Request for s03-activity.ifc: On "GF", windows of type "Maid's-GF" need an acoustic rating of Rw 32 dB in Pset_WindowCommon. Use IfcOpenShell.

First a look at what the model holds.

```python
import ifcopenshell
import ifcopenshell.util.element

model = ifcopenshell.open("s03-activity.ifc")
print(model.schema)
storey = next(s for s in model.by_type("IfcBuildingStorey") if s.Name == "GF")
windows = [e for e in ifcopenshell.util.element.get_decomposition(storey) if e.is_a("IfcWindow")]
seen = {}
for e in windows:
    element_type = ifcopenshell.util.element.get_type(e)
    key = (element_type.Name if element_type != e and element_type else None, ifcopenshell.util.element.get_pset(e, "Pset_WindowCommon", "AcousticRating"))
    seen[key] = seen.get(key, 0) + 1
for (name, value), count in sorted(seen.items(), key=str):
    print(count, "x", name, "|", value)
```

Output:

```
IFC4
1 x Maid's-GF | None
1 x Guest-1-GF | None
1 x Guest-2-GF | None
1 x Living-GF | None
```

```python
import ifcopenshell
import ifcopenshell.api.pset
import ifcopenshell.util.element

model = ifcopenshell.open("s03-activity.ifc")

storey = next(s for s in model.by_type("IfcBuildingStorey") if s.Name == "GF")
windows = [e for e in ifcopenshell.util.element.get_decomposition(storey) if e.is_a("IfcWindow")]

count = 0
for e in windows:
    element_type = ifcopenshell.util.element.get_type(e)
    if element_type in (None, e) or element_type.Name != "Maid's-GF":
        continue
    # add_pset returns the element's existing set when there is one.
    pset = ifcopenshell.api.pset.add_pset(model, product=e, name="Pset_WindowCommon")
    ifcopenshell.api.pset.edit_pset(model, pset=pset, properties={"AcousticRating": "Rw 32 dB"})
    count += 1

print(count, "windows updated")

model.write("s03-activity-out.ifc")
```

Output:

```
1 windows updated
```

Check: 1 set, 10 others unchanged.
